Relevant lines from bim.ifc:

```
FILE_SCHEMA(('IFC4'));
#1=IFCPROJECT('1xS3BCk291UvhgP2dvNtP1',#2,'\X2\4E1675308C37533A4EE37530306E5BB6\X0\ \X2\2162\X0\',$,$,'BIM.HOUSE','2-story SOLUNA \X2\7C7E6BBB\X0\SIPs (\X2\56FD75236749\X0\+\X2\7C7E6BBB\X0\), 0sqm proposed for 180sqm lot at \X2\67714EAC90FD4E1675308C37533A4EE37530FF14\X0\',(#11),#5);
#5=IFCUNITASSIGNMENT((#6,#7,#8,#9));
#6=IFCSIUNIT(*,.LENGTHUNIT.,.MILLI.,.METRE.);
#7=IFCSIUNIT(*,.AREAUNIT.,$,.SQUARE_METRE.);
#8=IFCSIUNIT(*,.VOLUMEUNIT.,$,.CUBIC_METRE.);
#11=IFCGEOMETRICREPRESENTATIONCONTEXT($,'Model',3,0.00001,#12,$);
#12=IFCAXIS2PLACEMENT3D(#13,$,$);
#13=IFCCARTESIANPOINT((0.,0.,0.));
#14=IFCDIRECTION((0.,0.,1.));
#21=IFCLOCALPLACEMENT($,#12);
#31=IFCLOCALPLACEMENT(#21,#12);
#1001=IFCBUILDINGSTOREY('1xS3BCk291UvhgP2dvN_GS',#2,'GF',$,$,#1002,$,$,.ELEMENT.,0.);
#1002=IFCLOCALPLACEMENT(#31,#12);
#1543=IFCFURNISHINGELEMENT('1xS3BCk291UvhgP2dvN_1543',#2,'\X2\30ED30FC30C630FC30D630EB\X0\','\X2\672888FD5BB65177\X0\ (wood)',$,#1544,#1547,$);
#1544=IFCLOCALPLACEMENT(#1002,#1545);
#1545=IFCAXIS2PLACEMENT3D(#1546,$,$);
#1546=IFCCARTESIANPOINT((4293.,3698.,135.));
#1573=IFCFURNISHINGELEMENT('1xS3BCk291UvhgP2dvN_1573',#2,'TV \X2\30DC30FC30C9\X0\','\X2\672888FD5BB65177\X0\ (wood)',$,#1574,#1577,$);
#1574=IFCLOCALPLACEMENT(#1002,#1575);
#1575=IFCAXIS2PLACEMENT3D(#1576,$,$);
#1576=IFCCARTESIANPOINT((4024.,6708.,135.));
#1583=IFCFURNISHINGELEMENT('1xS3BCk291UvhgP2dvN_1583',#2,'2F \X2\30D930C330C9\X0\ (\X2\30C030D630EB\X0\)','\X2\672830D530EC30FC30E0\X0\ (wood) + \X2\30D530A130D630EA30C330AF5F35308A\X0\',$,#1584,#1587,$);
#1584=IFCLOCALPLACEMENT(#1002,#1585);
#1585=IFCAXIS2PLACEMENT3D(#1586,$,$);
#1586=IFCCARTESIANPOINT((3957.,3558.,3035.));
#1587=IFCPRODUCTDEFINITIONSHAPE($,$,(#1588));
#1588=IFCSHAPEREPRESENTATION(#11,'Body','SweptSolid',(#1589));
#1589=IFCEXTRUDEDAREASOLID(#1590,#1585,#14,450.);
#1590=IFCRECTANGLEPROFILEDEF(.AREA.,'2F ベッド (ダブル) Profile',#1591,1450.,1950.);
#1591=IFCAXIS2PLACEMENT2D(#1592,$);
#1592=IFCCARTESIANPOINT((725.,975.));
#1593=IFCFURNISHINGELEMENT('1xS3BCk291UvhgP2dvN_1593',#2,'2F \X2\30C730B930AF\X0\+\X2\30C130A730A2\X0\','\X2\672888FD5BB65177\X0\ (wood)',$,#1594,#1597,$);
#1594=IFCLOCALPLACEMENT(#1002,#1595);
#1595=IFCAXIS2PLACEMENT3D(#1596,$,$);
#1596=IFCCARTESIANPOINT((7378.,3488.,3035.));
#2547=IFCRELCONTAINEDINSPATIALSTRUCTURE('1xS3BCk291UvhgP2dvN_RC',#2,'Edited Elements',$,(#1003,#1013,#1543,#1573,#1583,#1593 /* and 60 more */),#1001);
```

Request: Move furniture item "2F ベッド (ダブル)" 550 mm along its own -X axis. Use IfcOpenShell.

```python
import ifcopenshell
import ifcopenshell.api.geometry
import ifcopenshell.util.placement
import ifcopenshell.util.unit

model = ifcopenshell.open("bim.ifc")
unit_scale = ifcopenshell.util.unit.calculate_unit_scale(model)

item = model.by_guid("1xS3BCk291UvhgP2dvN_1583")
matrix = ifcopenshell.util.placement.get_local_placement(item.ObjectPlacement)
matrix[:3, 3] -= matrix[:3, 0] * 0.55 / unit_scale
ifcopenshell.api.geometry.edit_object_placement(model, product=item, matrix=matrix, is_si=False)

print(ifcopenshell.util.placement.get_local_placement(item.ObjectPlacement).round(3) + 0.0)

model.write("bim-out.ifc")
```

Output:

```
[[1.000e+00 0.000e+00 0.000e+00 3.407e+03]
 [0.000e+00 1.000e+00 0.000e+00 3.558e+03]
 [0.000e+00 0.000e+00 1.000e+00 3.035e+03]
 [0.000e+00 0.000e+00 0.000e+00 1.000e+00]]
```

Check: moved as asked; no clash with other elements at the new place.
